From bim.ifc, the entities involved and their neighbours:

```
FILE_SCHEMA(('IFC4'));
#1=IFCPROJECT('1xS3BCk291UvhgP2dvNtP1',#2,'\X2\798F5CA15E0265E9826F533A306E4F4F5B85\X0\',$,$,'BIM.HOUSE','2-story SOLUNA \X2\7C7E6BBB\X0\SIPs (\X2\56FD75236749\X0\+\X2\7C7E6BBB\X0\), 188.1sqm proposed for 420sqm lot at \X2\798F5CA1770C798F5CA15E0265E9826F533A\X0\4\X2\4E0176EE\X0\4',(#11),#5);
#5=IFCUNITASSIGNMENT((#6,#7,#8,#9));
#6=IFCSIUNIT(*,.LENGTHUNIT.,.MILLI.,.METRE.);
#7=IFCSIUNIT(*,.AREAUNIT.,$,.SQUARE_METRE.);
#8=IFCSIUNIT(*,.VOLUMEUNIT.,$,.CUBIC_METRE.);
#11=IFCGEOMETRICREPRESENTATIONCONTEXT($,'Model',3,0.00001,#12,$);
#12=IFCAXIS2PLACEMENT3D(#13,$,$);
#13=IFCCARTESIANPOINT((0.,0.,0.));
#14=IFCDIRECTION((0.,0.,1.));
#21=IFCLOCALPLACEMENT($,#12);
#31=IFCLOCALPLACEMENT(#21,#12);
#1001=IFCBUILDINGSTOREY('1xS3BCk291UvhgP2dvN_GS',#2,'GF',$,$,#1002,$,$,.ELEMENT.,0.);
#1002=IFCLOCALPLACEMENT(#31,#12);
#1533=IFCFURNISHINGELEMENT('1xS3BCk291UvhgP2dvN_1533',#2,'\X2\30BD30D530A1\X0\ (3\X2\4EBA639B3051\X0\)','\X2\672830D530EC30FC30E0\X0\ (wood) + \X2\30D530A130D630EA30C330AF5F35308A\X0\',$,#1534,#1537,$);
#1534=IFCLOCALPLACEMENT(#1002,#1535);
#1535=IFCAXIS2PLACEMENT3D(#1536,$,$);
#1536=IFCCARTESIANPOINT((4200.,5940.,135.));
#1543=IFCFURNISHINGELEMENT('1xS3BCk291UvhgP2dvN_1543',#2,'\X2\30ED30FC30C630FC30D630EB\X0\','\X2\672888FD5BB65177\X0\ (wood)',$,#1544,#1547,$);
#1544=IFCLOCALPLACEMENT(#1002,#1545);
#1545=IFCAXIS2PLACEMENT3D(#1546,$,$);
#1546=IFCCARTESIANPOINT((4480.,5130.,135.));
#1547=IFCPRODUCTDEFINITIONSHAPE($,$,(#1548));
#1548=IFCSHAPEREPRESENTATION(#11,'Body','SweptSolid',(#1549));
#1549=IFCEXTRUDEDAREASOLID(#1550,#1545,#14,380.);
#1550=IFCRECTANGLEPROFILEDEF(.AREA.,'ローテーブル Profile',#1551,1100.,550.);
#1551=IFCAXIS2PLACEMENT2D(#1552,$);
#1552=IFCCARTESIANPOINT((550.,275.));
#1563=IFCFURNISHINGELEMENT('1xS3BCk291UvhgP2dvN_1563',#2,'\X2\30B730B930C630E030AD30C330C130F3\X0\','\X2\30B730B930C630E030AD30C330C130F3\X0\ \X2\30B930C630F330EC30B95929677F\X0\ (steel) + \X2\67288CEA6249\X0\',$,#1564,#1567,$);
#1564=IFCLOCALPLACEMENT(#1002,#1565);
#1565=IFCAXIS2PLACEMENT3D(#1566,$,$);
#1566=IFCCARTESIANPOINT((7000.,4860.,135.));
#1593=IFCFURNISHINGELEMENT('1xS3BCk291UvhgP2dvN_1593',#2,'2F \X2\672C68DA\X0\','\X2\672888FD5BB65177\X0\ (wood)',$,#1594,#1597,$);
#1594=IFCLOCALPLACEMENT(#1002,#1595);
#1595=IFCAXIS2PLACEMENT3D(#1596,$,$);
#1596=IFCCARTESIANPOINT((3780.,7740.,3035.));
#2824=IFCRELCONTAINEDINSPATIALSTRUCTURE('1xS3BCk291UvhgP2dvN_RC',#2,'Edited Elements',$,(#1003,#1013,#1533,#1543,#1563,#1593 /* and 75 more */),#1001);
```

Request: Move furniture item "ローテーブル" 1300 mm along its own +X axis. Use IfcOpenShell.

```python
import ifcopenshell
import ifcopenshell.api.geometry
import ifcopenshell.util.placement
import ifcopenshell.util.unit

model = ifcopenshell.open("bim.ifc")
unit_scale = ifcopenshell.util.unit.calculate_unit_scale(model)

item = model.by_id(1543)
matrix = ifcopenshell.util.placement.get_local_placement(item.ObjectPlacement)
matrix[:3, 3] += matrix[:3, 0] * 1.3 / unit_scale
ifcopenshell.api.geometry.edit_object_placement(model, product=item, matrix=matrix, is_si=False)

print(ifcopenshell.util.placement.get_local_placement(item.ObjectPlacement).round(3) + 0.0)

model.write("bim_updated.ifc")
```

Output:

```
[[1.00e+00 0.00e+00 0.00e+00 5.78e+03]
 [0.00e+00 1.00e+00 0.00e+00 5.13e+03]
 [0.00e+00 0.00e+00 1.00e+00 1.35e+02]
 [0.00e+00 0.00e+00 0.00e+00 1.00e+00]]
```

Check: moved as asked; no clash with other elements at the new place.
